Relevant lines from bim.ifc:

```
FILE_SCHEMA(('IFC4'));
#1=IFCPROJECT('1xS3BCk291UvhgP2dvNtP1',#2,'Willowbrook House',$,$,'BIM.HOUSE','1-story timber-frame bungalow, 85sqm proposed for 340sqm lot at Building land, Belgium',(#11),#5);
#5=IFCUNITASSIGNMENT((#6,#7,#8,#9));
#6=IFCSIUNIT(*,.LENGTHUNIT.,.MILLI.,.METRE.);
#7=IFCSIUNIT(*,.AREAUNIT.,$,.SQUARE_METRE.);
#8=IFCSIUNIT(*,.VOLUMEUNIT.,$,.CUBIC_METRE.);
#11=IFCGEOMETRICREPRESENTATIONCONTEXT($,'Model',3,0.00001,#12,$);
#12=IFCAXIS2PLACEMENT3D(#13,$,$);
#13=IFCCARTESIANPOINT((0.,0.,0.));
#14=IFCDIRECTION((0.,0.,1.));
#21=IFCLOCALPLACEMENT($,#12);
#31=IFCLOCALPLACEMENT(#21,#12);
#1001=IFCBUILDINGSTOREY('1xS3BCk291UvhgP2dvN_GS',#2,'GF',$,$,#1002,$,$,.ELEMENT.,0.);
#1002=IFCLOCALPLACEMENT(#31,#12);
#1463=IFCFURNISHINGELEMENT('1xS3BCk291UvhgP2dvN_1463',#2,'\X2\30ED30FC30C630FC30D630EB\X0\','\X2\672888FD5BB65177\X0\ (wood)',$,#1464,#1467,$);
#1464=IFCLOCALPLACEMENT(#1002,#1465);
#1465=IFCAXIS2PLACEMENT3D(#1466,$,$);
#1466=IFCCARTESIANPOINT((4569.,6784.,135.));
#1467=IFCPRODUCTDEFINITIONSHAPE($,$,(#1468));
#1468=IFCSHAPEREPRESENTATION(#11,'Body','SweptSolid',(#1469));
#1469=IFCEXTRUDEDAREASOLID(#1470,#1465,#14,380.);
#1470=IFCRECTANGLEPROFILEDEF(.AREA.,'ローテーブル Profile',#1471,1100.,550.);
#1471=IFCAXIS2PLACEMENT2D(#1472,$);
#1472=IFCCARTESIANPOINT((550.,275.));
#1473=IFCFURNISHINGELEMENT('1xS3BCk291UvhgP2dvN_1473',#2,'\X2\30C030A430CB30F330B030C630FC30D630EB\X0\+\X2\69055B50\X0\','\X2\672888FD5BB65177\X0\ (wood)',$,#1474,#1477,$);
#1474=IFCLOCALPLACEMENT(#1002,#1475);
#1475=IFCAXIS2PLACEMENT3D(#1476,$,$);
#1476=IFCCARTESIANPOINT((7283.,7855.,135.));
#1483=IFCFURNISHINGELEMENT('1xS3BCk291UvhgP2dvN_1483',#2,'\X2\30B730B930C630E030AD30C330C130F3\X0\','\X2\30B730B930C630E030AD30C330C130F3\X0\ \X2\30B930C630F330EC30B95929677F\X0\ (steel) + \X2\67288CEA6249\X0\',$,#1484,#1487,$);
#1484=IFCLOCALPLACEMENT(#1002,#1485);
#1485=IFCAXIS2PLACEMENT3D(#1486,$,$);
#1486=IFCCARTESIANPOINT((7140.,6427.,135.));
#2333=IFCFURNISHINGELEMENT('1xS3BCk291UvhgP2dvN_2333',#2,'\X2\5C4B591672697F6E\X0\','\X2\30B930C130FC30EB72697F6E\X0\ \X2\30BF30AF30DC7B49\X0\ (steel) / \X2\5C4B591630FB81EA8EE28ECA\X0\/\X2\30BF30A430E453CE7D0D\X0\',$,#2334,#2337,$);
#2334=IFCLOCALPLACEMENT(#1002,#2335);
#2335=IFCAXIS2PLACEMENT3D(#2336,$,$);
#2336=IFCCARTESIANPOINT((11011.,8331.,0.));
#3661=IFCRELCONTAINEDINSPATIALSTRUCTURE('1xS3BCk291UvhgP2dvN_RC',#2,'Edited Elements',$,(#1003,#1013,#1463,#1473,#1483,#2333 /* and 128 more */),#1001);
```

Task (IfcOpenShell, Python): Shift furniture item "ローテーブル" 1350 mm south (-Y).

```python
import ifcopenshell
import ifcopenshell.api.geometry
import ifcopenshell.util.placement
import ifcopenshell.util.unit

model = ifcopenshell.open("bim.ifc")
unit_scale = ifcopenshell.util.unit.calculate_unit_scale(model)

item = model.by_id(1463)
matrix = ifcopenshell.util.placement.get_local_placement(item.ObjectPlacement)
matrix[1, 3] -= 1.35 / unit_scale
ifcopenshell.api.geometry.edit_object_placement(model, product=item, matrix=matrix, is_si=False)

print(ifcopenshell.util.placement.get_local_placement(item.ObjectPlacement).round(3) + 0.0)

model.write("bim-out.ifc")
```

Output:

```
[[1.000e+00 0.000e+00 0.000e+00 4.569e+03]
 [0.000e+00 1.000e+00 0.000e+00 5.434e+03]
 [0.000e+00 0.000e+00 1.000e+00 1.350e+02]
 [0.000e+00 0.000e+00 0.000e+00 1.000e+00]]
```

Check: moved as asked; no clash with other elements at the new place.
